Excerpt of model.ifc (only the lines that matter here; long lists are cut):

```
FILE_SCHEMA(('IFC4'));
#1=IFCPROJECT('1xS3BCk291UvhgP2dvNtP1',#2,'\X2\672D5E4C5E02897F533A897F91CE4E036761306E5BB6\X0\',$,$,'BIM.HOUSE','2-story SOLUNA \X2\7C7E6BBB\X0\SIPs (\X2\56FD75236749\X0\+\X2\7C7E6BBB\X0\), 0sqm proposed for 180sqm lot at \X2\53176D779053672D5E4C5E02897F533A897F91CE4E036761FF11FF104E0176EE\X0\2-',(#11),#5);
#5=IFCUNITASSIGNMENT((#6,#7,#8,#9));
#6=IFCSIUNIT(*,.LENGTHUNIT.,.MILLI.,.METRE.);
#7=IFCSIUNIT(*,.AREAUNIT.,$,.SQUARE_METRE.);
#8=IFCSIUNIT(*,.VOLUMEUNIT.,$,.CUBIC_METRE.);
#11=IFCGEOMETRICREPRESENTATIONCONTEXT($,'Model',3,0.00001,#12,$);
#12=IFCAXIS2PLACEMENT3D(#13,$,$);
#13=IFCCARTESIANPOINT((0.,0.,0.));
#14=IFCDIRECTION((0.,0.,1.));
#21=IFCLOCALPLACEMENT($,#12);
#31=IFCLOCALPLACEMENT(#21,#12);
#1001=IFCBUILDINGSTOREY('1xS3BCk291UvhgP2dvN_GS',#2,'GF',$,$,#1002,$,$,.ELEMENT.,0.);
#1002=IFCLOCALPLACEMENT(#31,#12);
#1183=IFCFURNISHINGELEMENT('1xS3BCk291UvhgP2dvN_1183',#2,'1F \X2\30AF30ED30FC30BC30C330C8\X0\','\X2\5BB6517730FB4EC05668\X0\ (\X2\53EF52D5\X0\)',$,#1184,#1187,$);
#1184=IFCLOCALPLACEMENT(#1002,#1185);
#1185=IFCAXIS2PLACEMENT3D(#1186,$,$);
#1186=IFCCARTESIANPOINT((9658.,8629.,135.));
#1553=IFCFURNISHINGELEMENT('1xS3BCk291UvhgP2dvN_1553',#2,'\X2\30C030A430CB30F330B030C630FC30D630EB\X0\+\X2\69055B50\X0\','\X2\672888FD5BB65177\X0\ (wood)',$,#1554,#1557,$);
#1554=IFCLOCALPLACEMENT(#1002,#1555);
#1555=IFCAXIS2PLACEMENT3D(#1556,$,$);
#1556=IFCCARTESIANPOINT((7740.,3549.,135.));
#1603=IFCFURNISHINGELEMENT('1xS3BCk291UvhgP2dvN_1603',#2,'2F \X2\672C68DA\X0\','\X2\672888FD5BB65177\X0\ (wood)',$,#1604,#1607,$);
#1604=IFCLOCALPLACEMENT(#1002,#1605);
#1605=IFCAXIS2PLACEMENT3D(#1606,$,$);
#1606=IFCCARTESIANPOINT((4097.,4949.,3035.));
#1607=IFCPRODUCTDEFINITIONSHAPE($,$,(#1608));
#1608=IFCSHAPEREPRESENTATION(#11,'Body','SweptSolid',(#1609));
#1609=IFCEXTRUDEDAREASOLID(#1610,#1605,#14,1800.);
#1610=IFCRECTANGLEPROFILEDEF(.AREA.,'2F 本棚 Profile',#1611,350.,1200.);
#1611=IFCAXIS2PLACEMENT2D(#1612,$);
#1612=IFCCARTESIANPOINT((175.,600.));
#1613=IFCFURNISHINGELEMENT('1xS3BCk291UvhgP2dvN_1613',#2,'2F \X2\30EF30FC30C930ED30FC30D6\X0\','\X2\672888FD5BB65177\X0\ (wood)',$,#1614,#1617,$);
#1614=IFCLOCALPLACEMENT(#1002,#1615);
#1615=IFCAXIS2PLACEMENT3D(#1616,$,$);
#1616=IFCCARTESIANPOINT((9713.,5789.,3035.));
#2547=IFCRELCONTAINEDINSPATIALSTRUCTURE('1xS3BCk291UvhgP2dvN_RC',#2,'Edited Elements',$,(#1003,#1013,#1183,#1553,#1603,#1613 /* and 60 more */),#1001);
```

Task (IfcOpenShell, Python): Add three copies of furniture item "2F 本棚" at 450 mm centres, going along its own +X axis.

```python
import ifcopenshell
import ifcopenshell.api.geometry
import ifcopenshell.api.root
import ifcopenshell.util.element
import ifcopenshell.util.placement
import ifcopenshell.util.unit

model = ifcopenshell.open("model.ifc")
unit_scale = ifcopenshell.util.unit.calculate_unit_scale(model)


def reuse_history(source, copy):
    """copy_class also copies each property set's owner history, people and application; keep the originals."""
    for rel in copy.IsDefinedBy:
        if rel.is_a("IfcRelDefinesByProperties") and (history := rel.RelatingPropertyDefinition.OwnerHistory):
            rel.RelatingPropertyDefinition.OwnerHistory = source.OwnerHistory
            ifcopenshell.util.element.remove_deep2(model, history)


source = model.by_id(1603)
base = ifcopenshell.util.placement.get_local_placement(source.ObjectPlacement)
step = base[:3, 0] * 0.45 / unit_scale

for i in range(1, 4):
    copy = ifcopenshell.api.root.copy_class(model, product=source)
    copy.Representation = ifcopenshell.util.element.copy_deep(
        model, source.Representation, exclude=["IfcGeometricRepresentationContext", "IfcRepresentationMap"]
    )
    reuse_history(source, copy)
    matrix = base.copy()
    matrix[:3, 3] += i * step
    print("added at", matrix[:3, 3].round(3) + 0.0)
    ifcopenshell.api.geometry.edit_object_placement(model, product=copy, matrix=matrix, is_si=False)

model.write("model-out.ifc")
```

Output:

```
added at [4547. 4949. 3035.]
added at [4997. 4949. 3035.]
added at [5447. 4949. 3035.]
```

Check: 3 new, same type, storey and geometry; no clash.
